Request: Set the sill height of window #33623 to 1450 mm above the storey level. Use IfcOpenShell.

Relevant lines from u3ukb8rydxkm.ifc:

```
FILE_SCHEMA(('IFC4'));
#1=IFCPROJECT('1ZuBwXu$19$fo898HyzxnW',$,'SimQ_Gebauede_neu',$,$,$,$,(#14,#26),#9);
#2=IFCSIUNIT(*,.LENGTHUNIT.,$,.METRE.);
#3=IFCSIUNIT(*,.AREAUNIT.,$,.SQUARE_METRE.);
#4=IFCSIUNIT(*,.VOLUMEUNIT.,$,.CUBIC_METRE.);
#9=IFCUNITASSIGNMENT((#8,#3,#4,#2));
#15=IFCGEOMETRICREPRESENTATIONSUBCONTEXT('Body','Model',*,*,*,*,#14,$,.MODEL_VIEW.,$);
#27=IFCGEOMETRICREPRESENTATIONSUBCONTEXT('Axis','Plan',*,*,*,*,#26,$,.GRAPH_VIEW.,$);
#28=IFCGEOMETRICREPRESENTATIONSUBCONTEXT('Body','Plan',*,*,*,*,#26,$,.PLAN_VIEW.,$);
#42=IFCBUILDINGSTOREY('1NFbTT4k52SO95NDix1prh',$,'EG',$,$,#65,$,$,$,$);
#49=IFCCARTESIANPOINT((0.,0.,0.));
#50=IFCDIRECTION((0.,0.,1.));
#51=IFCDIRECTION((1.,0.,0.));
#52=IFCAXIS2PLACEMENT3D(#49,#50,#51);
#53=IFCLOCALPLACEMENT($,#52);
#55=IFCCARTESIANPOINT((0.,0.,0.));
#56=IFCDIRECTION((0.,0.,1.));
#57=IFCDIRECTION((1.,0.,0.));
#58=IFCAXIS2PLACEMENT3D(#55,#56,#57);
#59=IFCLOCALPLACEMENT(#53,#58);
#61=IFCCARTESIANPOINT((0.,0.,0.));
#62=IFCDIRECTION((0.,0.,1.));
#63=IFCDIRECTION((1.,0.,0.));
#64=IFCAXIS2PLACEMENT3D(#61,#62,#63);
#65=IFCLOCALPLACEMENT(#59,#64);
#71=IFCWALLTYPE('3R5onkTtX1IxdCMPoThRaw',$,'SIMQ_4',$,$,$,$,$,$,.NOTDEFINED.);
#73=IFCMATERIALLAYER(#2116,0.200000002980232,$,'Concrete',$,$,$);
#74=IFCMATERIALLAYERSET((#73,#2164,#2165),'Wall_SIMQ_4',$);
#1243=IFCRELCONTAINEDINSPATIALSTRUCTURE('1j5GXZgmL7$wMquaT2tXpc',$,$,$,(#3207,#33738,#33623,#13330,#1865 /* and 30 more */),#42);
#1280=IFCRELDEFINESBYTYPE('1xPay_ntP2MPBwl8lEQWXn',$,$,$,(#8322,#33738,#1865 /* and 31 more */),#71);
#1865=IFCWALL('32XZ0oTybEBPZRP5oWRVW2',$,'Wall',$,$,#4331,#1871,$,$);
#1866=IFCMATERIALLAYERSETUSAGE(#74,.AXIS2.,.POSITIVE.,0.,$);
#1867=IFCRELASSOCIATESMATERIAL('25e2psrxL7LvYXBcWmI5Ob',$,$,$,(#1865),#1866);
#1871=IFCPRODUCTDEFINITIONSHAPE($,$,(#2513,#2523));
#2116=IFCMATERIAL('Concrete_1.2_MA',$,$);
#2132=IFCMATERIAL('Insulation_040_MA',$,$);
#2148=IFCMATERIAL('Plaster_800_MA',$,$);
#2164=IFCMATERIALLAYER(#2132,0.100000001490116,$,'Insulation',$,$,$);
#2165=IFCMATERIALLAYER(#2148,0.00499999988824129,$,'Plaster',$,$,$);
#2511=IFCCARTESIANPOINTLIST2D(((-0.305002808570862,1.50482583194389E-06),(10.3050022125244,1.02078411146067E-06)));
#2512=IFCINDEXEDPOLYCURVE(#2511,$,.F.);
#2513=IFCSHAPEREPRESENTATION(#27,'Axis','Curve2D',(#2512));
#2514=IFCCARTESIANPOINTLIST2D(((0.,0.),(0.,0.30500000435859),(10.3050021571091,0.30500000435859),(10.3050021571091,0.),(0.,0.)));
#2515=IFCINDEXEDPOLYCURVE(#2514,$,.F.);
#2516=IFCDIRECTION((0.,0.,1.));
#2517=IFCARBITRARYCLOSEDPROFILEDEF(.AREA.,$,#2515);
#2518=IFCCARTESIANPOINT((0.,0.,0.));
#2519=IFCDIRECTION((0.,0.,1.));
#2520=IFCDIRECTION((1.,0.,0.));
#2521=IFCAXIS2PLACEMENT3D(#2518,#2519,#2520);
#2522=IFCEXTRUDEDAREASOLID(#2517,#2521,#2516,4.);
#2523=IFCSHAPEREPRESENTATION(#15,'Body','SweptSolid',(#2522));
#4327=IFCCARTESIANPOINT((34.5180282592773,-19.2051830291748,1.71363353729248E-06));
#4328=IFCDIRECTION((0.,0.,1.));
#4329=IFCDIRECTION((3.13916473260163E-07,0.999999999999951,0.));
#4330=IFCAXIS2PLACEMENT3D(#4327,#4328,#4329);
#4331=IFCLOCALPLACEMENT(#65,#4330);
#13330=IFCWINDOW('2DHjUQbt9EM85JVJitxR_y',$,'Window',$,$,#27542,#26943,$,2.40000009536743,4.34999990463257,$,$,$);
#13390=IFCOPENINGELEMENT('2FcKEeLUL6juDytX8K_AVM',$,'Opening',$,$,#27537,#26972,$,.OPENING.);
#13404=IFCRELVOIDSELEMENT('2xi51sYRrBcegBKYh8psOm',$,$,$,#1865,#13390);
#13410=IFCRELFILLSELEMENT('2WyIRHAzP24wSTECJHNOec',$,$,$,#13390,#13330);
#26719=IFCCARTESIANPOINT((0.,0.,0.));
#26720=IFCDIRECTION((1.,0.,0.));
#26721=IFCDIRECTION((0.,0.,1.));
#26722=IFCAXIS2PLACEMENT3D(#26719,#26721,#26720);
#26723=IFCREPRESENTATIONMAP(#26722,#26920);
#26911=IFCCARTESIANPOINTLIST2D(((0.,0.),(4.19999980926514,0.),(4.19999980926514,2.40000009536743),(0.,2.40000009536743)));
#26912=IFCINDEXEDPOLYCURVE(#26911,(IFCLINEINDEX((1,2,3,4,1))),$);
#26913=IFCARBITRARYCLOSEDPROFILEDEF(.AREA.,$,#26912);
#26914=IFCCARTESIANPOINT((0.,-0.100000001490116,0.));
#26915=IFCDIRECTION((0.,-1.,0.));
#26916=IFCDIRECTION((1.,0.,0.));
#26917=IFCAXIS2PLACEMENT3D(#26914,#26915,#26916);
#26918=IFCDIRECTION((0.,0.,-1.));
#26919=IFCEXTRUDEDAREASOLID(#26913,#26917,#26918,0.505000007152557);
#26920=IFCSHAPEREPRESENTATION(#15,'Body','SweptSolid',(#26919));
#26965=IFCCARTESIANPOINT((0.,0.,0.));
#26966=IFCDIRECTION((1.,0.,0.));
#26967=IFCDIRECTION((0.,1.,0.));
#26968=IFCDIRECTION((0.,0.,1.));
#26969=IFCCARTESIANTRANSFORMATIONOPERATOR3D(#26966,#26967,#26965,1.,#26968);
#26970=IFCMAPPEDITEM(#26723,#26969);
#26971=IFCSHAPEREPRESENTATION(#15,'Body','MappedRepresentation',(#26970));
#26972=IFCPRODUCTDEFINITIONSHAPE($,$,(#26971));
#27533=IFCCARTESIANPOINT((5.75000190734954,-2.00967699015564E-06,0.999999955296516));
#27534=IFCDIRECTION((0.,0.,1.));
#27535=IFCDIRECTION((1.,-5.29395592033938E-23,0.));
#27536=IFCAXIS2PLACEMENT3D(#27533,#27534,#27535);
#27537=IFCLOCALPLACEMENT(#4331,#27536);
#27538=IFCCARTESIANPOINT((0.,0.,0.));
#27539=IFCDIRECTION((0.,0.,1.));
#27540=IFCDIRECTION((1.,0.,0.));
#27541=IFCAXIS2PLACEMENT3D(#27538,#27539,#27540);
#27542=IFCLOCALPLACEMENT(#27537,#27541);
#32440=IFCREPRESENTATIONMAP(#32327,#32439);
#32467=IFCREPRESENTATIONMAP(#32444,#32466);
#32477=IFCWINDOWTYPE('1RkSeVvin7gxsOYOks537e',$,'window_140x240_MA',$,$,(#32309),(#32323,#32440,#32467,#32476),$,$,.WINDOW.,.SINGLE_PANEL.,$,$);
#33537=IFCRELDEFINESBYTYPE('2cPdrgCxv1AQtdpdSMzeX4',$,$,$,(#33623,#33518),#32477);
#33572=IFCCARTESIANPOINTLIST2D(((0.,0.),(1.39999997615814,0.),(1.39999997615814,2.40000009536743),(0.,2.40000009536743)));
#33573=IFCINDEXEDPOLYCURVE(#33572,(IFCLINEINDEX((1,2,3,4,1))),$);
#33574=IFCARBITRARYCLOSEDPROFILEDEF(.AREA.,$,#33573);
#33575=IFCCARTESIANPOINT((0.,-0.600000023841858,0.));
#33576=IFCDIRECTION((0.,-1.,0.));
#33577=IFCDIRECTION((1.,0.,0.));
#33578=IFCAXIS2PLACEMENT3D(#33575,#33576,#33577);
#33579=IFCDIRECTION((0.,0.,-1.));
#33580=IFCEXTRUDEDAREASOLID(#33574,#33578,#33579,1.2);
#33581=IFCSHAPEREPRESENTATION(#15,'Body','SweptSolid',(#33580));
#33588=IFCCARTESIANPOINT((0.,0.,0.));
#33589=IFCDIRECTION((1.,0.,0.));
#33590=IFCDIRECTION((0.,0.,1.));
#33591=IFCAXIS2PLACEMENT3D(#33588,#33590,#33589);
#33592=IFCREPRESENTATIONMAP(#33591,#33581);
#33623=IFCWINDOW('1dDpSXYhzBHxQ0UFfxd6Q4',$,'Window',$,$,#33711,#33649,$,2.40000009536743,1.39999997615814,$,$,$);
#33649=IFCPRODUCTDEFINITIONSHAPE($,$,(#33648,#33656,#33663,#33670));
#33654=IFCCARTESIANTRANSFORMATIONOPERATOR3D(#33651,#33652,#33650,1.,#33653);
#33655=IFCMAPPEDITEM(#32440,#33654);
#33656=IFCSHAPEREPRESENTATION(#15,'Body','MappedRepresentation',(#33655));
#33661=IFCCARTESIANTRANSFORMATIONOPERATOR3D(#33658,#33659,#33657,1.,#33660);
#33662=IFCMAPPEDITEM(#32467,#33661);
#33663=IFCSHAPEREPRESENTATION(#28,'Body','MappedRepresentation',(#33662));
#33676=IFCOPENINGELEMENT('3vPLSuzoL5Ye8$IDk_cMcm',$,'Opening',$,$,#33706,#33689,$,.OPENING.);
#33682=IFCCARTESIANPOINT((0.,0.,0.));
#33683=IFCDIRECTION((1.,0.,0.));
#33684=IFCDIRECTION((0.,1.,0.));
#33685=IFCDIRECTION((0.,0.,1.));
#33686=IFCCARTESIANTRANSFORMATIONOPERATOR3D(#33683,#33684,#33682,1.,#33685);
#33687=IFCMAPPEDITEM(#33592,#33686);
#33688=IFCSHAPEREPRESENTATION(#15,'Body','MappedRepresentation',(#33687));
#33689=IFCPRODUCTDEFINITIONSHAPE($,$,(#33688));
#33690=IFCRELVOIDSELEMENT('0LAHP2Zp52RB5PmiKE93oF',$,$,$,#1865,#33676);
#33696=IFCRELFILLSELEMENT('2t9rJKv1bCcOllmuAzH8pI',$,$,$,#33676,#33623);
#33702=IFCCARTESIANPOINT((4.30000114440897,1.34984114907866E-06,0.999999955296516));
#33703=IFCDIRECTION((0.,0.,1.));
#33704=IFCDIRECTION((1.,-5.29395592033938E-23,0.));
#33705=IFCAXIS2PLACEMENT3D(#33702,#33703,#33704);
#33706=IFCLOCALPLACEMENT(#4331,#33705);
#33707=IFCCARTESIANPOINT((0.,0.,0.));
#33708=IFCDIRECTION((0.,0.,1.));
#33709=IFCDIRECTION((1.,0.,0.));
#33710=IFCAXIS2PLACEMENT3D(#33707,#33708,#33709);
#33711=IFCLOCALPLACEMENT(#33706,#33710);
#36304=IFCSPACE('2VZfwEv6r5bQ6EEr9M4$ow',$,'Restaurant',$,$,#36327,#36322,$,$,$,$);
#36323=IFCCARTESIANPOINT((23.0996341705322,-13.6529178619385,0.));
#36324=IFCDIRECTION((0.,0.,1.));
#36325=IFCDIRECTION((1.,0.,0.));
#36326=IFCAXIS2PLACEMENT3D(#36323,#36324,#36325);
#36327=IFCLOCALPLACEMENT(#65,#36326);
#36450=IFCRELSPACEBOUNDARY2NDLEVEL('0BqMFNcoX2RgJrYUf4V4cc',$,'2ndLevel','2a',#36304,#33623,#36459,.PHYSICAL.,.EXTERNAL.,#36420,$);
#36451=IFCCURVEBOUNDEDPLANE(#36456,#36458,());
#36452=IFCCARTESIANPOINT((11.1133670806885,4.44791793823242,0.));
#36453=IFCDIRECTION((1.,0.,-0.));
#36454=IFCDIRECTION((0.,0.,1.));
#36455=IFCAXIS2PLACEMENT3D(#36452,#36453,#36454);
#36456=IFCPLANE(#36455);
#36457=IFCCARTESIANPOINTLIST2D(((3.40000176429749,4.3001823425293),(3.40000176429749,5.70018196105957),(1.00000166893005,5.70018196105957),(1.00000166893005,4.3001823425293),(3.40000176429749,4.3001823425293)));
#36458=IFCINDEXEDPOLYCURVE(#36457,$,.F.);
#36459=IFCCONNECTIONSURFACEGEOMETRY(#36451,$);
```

```python
import numpy as np
import ifcopenshell
import ifcopenshell.api.geometry
import ifcopenshell.geom
import ifcopenshell.util.element
import ifcopenshell.util.placement
import ifcopenshell.util.shape
import ifcopenshell.util.unit

model = ifcopenshell.open("u3ukb8rydxkm.ifc")
unit_scale = ifcopenshell.util.unit.calculate_unit_scale(model)

window = model.by_guid("1dDpSXYhzBHxQ0UFfxd6Q4")
opening = window.FillsVoids[0].RelatingOpeningElement
storey = ifcopenshell.util.element.get_container(window, ifc_class="IfcBuildingStorey")
level = ifcopenshell.util.placement.get_local_placement(storey.ObjectPlacement)[2, 3]

# The opening's origin need not be at the sill, so measure its lowest point.
shape = ifcopenshell.geom.create_shape(ifcopenshell.geom.settings(), opening)
bottom = ifcopenshell.util.shape.get_shape_bottom_elevation(shape, shape.geometry) / unit_scale
dz = level + 1.45 - bottom

shift = np.array([0.0, 0.0, dz])
# The window is placed relative to its opening, so it follows when the opening moves.
matrix = ifcopenshell.util.placement.get_local_placement(opening.ObjectPlacement)
matrix[:3, 3] += shift
ifcopenshell.api.geometry.edit_object_placement(
    model, product=opening, matrix=matrix, is_si=False, should_transform_children=True
)

# Space boundary surfaces are stored in each space's coordinates; move them too.
for rel in window.ProvidesBoundaries:
    if not rel.ConnectionGeometry:
        continue
    surface = rel.ConnectionGeometry.SurfaceOnRelatingElement.BasisSurface
    space_matrix = ifcopenshell.util.placement.get_local_placement(rel.RelatingSpace.ObjectPlacement)
    point = np.array(surface.Position.Location.Coordinates) + space_matrix[:3, :3].T @ shift
    surface.Position = model.createIfcAxis2Placement3D(
        model.createIfcCartesianPoint(point.tolist()), surface.Position.Axis, surface.Position.RefDirection
    )

print(f"moved by {dz * unit_scale:+.3f} m")

model.write("u3ukb8rydxkm_edited.ifc")
```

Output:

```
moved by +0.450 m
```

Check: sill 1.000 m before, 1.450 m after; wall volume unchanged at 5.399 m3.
